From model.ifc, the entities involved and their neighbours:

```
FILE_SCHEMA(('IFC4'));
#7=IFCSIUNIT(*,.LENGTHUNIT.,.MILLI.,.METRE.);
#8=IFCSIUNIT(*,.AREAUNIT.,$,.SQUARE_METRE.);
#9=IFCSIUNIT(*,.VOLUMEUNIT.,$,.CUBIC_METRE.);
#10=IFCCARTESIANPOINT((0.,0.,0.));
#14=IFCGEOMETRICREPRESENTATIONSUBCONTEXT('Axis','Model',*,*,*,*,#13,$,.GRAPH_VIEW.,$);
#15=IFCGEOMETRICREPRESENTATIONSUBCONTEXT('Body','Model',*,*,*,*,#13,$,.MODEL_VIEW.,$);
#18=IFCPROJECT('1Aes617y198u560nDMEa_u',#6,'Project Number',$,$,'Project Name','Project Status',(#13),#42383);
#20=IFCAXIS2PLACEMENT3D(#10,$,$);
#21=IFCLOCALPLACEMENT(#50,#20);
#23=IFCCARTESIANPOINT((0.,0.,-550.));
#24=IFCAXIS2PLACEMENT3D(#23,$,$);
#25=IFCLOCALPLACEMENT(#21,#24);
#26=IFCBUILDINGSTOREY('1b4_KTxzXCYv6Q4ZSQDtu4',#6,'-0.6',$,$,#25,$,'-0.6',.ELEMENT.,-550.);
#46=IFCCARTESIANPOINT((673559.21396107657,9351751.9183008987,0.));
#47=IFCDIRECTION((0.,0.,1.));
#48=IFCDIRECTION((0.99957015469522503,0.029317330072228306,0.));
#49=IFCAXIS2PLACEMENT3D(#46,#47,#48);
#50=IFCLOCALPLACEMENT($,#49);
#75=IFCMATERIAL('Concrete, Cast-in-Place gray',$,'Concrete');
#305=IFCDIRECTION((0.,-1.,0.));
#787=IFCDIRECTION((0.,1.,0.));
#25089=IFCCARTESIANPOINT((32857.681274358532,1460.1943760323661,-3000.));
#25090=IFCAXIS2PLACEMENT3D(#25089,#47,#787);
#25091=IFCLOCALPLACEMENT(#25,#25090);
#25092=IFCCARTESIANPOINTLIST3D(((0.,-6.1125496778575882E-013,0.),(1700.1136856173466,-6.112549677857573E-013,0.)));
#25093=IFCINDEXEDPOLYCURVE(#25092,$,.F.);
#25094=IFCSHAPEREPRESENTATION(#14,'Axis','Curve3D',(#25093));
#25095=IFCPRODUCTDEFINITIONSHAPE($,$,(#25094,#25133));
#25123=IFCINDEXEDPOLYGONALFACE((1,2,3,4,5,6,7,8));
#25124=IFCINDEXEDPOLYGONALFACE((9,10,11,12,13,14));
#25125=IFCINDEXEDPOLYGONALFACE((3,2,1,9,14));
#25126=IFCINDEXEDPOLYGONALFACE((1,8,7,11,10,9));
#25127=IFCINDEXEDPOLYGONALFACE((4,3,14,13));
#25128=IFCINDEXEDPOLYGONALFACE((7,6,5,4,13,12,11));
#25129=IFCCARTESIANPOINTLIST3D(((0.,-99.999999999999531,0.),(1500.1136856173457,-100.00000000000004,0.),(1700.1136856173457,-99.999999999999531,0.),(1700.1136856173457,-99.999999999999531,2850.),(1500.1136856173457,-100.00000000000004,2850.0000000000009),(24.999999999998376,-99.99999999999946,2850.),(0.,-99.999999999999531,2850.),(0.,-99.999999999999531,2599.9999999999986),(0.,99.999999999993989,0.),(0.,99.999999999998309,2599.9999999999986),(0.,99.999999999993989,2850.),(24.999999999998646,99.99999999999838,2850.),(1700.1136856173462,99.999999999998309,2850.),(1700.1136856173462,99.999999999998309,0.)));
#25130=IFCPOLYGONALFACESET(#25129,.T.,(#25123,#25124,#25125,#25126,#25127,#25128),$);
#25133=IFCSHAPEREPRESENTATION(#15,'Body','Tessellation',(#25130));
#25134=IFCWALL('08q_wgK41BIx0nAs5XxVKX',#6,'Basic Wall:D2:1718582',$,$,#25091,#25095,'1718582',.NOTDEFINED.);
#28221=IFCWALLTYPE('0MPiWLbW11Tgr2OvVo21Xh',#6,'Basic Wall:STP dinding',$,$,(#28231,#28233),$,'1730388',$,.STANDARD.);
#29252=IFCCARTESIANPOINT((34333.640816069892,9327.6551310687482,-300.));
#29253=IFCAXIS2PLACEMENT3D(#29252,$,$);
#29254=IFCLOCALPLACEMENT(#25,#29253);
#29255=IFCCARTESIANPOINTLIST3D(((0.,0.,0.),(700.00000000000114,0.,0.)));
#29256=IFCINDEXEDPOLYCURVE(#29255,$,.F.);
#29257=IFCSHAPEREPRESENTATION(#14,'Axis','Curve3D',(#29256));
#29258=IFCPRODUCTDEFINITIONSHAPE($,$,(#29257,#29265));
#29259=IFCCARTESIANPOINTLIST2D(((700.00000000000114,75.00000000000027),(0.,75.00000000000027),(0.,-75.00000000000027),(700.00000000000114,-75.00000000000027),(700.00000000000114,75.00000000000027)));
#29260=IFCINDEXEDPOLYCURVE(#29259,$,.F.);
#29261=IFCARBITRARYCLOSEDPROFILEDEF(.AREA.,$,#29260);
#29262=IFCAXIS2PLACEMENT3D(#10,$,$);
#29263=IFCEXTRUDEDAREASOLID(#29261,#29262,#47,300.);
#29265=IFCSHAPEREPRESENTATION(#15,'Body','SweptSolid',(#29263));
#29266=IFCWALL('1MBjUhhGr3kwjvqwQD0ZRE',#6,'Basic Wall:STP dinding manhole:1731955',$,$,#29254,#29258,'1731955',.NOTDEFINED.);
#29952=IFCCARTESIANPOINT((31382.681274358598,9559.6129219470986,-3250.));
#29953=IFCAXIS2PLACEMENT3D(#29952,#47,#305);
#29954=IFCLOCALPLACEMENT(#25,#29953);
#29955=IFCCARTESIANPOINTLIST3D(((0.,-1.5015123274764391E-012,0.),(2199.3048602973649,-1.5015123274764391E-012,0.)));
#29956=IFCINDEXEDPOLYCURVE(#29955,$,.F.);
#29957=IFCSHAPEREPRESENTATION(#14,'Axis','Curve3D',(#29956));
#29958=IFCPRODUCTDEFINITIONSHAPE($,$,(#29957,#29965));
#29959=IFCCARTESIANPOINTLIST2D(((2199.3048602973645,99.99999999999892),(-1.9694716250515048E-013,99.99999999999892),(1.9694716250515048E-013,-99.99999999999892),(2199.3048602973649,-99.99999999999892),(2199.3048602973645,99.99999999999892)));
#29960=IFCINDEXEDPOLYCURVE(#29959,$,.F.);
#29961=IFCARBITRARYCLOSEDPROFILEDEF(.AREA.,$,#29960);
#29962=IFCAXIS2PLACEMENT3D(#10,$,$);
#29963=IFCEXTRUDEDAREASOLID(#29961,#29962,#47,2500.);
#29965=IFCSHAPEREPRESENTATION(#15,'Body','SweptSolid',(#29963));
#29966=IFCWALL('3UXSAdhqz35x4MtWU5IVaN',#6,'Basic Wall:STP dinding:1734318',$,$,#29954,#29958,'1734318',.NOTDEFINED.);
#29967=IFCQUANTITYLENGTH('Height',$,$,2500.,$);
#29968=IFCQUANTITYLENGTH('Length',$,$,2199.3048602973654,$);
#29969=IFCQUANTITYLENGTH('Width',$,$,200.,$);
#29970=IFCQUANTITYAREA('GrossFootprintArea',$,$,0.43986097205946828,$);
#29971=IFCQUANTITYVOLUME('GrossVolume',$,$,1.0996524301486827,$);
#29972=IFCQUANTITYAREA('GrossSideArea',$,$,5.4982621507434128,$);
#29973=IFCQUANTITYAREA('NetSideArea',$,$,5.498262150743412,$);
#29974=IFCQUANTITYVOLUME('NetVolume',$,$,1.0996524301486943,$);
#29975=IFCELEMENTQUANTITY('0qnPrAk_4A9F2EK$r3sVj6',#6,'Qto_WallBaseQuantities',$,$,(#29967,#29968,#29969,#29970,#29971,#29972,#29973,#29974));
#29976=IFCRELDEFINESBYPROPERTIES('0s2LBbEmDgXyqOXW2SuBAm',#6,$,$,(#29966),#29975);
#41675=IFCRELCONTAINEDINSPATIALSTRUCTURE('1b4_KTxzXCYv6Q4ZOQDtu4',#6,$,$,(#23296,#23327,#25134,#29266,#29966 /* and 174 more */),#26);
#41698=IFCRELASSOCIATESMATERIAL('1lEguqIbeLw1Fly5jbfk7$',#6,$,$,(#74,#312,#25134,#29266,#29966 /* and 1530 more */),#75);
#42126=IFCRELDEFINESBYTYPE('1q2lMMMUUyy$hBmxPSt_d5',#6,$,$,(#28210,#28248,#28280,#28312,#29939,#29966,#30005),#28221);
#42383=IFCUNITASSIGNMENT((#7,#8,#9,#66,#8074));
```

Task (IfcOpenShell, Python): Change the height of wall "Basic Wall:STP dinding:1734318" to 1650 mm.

```python
import ifcopenshell
import ifcopenshell.api.pset
import ifcopenshell.geom
import ifcopenshell.util.element
import ifcopenshell.util.representation
import ifcopenshell.util.shape
import ifcopenshell.util.unit

model = ifcopenshell.open("model.ifc")
unit_scale = ifcopenshell.util.unit.calculate_unit_scale(model)
area_scale = ifcopenshell.util.unit.calculate_unit_scale(model, "AREAUNIT")
volume_scale = ifcopenshell.util.unit.calculate_unit_scale(model, "VOLUMEUNIT")
settings = ifcopenshell.geom.settings()


def volume(element):
    """Net volume in cubic metres, openings subtracted."""
    shape = ifcopenshell.geom.create_shape(settings, element)
    return ifcopenshell.util.shape.get_volume(shape.geometry)


wall = model.by_id(29966)
before = volume(wall)

body = ifcopenshell.util.representation.get_representation(wall, "Model", "Body")
solid = body.Items[0]
old_height = solid.Depth
solid.Depth = 1.65 / unit_scale
after = volume(wall)
thickness = 0.2  # wall thickness in metres

# Update the stored height, areas and volumes.
qto = model.by_id(ifcopenshell.util.element.get_pset(wall, "Qto_WallBaseQuantities", should_inherit=False)["id"])
ifcopenshell.api.pset.edit_qto(model, qto=qto, properties={
    "Height": solid.Depth,
    "GrossVolume": ifcopenshell.util.element.get_pset(wall, "Qto_WallBaseQuantities", "GrossVolume") * solid.Depth / old_height,
    "GrossSideArea": ifcopenshell.util.element.get_pset(wall, "Qto_WallBaseQuantities", "GrossSideArea") * solid.Depth / old_height,
    "NetSideArea": after / thickness / area_scale,
    "NetVolume": after / volume_scale,
})

print(f"height {old_height:g} -> {solid.Depth:g}, volume {before:.3f} -> {after:.3f} m3")

model.write("model_rev.ifc")
```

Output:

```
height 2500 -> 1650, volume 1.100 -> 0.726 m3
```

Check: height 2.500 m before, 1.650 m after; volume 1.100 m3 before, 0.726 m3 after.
